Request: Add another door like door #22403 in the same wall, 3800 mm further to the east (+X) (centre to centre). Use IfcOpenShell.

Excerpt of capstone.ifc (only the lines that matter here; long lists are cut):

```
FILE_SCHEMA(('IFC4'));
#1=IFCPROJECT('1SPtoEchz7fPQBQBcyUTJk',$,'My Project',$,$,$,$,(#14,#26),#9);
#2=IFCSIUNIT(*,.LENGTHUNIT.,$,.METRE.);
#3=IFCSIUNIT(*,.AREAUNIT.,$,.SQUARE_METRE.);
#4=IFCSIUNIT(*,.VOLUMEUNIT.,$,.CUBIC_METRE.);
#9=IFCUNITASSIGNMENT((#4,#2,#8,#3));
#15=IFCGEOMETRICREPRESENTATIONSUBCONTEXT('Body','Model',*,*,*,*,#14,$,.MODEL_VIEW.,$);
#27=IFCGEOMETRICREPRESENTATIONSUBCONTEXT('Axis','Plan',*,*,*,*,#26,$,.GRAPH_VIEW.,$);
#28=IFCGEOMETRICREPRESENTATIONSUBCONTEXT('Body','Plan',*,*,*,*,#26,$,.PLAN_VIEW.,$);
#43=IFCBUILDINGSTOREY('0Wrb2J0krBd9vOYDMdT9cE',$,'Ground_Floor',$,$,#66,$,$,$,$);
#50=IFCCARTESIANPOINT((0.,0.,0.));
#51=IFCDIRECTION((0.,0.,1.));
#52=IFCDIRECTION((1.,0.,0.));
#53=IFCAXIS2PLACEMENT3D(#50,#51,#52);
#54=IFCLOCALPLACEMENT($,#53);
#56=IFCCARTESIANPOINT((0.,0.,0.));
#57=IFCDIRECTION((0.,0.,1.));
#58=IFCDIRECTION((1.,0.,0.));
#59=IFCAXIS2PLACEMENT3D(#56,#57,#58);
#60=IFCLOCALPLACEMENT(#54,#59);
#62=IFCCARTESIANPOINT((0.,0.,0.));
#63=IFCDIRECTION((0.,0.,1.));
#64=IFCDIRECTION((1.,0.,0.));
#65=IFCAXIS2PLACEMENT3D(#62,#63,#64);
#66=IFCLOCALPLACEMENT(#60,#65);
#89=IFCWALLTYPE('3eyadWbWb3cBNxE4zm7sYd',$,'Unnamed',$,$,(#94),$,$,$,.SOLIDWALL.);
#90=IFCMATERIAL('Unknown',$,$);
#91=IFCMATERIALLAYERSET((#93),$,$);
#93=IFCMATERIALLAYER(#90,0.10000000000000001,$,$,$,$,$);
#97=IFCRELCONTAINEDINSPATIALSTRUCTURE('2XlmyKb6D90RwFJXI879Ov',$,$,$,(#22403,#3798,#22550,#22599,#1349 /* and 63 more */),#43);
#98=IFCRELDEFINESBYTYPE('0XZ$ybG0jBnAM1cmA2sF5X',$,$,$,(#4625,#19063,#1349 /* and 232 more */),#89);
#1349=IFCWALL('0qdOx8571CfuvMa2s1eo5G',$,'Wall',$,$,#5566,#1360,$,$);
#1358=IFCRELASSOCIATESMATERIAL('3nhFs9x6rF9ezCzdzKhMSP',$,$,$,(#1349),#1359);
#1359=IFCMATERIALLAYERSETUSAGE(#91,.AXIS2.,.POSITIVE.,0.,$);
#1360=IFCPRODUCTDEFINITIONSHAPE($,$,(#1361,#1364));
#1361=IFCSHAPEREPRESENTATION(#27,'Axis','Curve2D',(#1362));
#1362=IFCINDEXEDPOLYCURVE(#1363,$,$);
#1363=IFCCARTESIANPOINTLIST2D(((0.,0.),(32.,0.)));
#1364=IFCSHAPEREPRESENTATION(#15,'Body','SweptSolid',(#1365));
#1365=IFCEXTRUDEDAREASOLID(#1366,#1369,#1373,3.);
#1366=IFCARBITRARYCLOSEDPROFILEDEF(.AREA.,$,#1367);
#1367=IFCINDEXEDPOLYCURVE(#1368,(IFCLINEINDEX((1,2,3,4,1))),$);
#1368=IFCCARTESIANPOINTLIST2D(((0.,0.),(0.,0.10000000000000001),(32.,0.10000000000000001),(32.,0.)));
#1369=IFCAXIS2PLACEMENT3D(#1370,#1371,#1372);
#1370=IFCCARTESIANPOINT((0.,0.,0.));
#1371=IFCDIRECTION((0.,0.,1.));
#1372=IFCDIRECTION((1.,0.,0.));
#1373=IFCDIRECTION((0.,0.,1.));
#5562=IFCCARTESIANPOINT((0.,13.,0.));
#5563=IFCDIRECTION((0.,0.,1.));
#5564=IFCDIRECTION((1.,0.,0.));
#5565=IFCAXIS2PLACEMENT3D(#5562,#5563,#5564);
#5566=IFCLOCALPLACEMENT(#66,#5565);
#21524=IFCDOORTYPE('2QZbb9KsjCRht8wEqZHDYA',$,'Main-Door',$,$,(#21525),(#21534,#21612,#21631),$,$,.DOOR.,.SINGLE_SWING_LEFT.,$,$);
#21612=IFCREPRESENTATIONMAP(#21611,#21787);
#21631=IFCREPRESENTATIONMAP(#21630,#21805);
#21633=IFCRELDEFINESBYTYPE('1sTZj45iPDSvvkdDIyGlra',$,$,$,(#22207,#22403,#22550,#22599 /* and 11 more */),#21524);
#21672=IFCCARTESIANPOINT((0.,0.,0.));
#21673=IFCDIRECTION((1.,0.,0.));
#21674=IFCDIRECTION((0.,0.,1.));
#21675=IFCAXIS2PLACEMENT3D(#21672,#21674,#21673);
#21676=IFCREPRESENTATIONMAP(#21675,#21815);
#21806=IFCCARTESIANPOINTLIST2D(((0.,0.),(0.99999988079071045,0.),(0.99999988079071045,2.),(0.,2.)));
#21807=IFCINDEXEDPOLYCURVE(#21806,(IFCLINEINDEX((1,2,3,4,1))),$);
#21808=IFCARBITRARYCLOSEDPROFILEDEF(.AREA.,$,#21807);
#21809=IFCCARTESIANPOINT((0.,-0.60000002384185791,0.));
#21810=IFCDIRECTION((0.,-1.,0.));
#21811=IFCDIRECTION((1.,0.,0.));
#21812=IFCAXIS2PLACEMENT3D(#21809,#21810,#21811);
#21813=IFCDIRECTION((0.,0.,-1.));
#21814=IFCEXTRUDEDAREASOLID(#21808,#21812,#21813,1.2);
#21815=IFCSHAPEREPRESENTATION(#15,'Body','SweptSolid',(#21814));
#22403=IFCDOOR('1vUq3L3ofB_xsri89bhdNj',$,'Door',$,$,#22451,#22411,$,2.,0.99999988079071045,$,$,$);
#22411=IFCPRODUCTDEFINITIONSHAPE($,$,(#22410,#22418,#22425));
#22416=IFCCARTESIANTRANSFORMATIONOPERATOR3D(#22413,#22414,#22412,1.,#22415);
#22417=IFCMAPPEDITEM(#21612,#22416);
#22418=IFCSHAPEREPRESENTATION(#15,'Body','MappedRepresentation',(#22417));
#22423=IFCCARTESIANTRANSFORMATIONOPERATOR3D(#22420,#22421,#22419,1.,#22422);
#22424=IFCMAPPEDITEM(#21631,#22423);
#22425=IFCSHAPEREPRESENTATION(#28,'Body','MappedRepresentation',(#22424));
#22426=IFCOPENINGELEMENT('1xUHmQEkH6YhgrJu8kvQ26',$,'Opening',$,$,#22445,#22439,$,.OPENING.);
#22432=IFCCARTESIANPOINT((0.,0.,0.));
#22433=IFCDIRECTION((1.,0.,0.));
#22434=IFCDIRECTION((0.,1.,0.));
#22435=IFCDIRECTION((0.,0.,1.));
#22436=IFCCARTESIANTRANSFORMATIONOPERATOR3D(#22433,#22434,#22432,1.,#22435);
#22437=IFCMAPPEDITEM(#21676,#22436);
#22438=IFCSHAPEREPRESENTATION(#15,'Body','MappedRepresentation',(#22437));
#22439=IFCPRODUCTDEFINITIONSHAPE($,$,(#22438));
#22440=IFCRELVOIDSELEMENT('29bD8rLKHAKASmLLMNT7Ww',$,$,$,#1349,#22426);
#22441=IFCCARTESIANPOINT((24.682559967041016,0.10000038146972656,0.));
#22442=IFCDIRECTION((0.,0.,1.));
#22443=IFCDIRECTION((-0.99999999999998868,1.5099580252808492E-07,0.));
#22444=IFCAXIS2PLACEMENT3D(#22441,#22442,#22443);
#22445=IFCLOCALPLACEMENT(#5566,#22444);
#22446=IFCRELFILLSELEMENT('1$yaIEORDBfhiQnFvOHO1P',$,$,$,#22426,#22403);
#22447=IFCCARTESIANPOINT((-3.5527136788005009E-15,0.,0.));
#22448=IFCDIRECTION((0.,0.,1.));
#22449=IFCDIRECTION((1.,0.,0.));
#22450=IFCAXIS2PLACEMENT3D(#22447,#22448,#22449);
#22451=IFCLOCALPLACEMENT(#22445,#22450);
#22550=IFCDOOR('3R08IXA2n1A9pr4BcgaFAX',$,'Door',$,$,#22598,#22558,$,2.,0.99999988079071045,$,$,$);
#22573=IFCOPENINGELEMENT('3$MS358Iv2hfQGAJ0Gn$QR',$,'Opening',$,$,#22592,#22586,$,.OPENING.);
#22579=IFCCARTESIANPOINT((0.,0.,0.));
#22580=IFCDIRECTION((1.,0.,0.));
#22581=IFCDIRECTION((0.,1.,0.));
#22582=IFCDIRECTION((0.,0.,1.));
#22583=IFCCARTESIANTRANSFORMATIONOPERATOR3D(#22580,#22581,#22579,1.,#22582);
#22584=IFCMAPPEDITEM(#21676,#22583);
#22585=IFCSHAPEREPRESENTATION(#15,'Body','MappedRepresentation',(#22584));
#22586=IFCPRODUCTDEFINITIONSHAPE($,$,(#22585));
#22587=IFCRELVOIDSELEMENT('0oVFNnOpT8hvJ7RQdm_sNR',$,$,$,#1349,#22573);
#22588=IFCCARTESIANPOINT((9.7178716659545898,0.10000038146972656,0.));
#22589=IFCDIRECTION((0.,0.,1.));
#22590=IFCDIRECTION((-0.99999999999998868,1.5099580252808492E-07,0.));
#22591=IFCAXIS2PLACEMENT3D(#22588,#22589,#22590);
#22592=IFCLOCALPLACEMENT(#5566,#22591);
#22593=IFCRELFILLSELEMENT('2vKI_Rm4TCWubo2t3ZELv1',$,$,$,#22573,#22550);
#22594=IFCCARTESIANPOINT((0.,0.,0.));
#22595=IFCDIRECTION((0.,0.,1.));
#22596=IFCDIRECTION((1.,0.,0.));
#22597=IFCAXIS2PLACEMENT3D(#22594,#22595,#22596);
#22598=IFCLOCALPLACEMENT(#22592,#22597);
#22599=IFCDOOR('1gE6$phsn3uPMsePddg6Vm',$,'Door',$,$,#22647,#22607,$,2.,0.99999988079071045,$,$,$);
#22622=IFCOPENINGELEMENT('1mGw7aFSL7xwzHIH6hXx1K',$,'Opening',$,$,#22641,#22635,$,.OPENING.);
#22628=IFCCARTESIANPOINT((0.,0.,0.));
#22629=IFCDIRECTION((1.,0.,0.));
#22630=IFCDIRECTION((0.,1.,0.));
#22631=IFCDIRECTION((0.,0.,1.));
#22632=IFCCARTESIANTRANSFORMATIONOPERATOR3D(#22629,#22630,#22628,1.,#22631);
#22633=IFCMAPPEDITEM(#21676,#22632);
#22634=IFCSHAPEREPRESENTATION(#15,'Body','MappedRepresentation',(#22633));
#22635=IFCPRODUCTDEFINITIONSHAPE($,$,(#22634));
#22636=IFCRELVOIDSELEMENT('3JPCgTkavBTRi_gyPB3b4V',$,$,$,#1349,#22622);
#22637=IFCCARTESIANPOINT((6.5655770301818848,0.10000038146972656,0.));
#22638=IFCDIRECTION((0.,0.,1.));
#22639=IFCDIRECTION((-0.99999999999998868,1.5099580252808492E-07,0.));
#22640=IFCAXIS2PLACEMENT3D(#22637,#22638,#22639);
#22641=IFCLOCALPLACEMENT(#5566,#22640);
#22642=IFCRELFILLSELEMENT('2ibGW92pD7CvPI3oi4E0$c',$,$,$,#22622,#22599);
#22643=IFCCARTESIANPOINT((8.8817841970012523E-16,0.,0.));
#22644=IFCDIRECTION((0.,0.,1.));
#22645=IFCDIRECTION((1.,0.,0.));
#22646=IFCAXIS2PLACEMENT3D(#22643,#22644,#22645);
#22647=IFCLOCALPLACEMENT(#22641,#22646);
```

```python
import ifcopenshell
import ifcopenshell.api.feature
import ifcopenshell.api.geometry
import ifcopenshell.api.root
import ifcopenshell.geom
import ifcopenshell.util.element
import ifcopenshell.util.placement
import ifcopenshell.util.shape
import ifcopenshell.util.unit

model = ifcopenshell.open("capstone.ifc")
unit_scale = ifcopenshell.util.unit.calculate_unit_scale(model)
settings = ifcopenshell.geom.settings()


def volume(element):
    """Net volume in cubic metres, openings subtracted."""
    shape = ifcopenshell.geom.create_shape(settings, element)
    return ifcopenshell.util.shape.get_volume(shape.geometry)


door = model.by_id(22403)
opening = door.FillsVoids[0].RelatingOpeningElement
wall = opening.VoidsElements[0].RelatingBuildingElement
before = volume(wall)
shift = ifcopenshell.util.placement.get_local_placement(wall.ObjectPlacement)[:3, 0] * 3.8 / unit_scale

# copy_class copies the void relationship, type, container and properties, but no geometry.
new_opening = ifcopenshell.api.root.copy_class(model, product=opening)
new_opening.Representation = ifcopenshell.util.element.copy_deep(
    model, opening.Representation, exclude=["IfcGeometricRepresentationContext", "IfcRepresentationMap"]
)
new_door = ifcopenshell.api.root.copy_class(model, product=door)
new_door.Representation = ifcopenshell.util.element.copy_deep(
    model, door.Representation, exclude=["IfcGeometricRepresentationContext", "IfcRepresentationMap"]
)
ifcopenshell.api.feature.add_filling(model, opening=new_opening, element=new_door)

for old, new in ((opening, new_opening), (door, new_door)):
    matrix = ifcopenshell.util.placement.get_local_placement(old.ObjectPlacement)
    matrix[:3, 3] += shift
    ifcopenshell.api.geometry.edit_object_placement(model, product=new, matrix=matrix, is_si=False)

after = volume(wall)

print(f"wall volume {before:.3f} -> {after:.3f} m3")

model.write("capstone_v2.ifc")
```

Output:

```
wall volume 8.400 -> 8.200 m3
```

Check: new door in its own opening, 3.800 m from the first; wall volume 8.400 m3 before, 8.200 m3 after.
